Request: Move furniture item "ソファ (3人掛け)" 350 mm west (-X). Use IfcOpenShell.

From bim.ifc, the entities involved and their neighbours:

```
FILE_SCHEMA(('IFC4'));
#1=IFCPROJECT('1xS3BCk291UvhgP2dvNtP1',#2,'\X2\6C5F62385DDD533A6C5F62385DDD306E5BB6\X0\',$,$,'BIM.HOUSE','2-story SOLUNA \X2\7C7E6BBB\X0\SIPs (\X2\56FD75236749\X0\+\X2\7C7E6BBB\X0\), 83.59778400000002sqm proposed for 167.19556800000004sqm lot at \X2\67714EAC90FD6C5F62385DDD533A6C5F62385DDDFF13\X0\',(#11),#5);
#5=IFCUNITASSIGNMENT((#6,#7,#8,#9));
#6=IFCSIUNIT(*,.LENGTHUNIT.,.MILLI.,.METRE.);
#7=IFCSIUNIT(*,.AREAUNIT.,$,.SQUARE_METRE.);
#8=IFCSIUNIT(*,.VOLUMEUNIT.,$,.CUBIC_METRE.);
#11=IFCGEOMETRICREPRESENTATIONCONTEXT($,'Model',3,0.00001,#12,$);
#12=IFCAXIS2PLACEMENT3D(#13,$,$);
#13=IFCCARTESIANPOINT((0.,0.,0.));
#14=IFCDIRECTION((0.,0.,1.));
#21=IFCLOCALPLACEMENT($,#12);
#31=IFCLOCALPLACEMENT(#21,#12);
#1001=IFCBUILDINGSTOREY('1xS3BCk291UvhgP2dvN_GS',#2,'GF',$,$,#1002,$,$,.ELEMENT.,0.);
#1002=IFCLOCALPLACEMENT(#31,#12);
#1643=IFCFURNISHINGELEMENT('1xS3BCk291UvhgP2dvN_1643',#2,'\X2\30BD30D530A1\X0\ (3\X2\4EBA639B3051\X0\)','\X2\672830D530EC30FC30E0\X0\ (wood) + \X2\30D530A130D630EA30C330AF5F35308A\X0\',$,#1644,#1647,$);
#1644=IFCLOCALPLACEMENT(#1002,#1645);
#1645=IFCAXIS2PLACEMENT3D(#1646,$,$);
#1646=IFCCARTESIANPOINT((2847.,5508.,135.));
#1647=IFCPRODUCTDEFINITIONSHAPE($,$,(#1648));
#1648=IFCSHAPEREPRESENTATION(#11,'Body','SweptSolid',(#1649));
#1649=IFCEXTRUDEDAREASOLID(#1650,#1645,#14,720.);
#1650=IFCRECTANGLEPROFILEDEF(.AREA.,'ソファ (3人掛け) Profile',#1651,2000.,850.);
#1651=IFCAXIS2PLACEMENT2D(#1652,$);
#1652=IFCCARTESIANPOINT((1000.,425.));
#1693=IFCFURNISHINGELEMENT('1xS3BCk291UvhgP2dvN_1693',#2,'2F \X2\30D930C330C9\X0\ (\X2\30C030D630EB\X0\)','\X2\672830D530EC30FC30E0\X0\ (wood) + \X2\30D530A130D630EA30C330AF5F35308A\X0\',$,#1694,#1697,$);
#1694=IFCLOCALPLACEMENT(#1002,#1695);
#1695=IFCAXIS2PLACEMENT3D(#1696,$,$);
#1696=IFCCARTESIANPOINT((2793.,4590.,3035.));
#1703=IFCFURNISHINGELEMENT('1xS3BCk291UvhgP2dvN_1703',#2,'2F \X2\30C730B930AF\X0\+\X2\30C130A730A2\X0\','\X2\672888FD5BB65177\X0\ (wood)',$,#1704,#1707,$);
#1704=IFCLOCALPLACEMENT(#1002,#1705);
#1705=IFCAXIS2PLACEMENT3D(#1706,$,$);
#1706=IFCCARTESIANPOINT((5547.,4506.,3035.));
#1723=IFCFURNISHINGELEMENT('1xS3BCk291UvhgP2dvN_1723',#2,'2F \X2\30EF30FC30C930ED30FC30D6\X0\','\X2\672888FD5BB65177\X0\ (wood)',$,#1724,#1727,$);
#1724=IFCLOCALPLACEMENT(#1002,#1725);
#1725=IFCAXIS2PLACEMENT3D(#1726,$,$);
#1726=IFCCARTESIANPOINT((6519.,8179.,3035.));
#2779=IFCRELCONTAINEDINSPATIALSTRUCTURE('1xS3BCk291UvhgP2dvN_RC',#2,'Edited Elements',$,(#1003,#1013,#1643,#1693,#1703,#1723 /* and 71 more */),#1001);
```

```python
import ifcopenshell
import ifcopenshell.api.geometry
import ifcopenshell.util.placement

model = ifcopenshell.open("bim.ifc")

item = model.by_guid("1xS3BCk291UvhgP2dvN_1643")
matrix = ifcopenshell.util.placement.get_local_placement(item.ObjectPlacement)
matrix[0, 3] -= 350.0
ifcopenshell.api.geometry.edit_object_placement(model, product=item, matrix=matrix, is_si=False)

print(ifcopenshell.util.placement.get_local_placement(item.ObjectPlacement).round(3) + 0.0)

model.write("bim_rev.ifc")
```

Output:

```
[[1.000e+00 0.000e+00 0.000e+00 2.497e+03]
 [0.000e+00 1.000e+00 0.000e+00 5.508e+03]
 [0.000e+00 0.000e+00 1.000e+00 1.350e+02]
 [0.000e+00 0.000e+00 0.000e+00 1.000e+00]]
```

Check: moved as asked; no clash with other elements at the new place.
